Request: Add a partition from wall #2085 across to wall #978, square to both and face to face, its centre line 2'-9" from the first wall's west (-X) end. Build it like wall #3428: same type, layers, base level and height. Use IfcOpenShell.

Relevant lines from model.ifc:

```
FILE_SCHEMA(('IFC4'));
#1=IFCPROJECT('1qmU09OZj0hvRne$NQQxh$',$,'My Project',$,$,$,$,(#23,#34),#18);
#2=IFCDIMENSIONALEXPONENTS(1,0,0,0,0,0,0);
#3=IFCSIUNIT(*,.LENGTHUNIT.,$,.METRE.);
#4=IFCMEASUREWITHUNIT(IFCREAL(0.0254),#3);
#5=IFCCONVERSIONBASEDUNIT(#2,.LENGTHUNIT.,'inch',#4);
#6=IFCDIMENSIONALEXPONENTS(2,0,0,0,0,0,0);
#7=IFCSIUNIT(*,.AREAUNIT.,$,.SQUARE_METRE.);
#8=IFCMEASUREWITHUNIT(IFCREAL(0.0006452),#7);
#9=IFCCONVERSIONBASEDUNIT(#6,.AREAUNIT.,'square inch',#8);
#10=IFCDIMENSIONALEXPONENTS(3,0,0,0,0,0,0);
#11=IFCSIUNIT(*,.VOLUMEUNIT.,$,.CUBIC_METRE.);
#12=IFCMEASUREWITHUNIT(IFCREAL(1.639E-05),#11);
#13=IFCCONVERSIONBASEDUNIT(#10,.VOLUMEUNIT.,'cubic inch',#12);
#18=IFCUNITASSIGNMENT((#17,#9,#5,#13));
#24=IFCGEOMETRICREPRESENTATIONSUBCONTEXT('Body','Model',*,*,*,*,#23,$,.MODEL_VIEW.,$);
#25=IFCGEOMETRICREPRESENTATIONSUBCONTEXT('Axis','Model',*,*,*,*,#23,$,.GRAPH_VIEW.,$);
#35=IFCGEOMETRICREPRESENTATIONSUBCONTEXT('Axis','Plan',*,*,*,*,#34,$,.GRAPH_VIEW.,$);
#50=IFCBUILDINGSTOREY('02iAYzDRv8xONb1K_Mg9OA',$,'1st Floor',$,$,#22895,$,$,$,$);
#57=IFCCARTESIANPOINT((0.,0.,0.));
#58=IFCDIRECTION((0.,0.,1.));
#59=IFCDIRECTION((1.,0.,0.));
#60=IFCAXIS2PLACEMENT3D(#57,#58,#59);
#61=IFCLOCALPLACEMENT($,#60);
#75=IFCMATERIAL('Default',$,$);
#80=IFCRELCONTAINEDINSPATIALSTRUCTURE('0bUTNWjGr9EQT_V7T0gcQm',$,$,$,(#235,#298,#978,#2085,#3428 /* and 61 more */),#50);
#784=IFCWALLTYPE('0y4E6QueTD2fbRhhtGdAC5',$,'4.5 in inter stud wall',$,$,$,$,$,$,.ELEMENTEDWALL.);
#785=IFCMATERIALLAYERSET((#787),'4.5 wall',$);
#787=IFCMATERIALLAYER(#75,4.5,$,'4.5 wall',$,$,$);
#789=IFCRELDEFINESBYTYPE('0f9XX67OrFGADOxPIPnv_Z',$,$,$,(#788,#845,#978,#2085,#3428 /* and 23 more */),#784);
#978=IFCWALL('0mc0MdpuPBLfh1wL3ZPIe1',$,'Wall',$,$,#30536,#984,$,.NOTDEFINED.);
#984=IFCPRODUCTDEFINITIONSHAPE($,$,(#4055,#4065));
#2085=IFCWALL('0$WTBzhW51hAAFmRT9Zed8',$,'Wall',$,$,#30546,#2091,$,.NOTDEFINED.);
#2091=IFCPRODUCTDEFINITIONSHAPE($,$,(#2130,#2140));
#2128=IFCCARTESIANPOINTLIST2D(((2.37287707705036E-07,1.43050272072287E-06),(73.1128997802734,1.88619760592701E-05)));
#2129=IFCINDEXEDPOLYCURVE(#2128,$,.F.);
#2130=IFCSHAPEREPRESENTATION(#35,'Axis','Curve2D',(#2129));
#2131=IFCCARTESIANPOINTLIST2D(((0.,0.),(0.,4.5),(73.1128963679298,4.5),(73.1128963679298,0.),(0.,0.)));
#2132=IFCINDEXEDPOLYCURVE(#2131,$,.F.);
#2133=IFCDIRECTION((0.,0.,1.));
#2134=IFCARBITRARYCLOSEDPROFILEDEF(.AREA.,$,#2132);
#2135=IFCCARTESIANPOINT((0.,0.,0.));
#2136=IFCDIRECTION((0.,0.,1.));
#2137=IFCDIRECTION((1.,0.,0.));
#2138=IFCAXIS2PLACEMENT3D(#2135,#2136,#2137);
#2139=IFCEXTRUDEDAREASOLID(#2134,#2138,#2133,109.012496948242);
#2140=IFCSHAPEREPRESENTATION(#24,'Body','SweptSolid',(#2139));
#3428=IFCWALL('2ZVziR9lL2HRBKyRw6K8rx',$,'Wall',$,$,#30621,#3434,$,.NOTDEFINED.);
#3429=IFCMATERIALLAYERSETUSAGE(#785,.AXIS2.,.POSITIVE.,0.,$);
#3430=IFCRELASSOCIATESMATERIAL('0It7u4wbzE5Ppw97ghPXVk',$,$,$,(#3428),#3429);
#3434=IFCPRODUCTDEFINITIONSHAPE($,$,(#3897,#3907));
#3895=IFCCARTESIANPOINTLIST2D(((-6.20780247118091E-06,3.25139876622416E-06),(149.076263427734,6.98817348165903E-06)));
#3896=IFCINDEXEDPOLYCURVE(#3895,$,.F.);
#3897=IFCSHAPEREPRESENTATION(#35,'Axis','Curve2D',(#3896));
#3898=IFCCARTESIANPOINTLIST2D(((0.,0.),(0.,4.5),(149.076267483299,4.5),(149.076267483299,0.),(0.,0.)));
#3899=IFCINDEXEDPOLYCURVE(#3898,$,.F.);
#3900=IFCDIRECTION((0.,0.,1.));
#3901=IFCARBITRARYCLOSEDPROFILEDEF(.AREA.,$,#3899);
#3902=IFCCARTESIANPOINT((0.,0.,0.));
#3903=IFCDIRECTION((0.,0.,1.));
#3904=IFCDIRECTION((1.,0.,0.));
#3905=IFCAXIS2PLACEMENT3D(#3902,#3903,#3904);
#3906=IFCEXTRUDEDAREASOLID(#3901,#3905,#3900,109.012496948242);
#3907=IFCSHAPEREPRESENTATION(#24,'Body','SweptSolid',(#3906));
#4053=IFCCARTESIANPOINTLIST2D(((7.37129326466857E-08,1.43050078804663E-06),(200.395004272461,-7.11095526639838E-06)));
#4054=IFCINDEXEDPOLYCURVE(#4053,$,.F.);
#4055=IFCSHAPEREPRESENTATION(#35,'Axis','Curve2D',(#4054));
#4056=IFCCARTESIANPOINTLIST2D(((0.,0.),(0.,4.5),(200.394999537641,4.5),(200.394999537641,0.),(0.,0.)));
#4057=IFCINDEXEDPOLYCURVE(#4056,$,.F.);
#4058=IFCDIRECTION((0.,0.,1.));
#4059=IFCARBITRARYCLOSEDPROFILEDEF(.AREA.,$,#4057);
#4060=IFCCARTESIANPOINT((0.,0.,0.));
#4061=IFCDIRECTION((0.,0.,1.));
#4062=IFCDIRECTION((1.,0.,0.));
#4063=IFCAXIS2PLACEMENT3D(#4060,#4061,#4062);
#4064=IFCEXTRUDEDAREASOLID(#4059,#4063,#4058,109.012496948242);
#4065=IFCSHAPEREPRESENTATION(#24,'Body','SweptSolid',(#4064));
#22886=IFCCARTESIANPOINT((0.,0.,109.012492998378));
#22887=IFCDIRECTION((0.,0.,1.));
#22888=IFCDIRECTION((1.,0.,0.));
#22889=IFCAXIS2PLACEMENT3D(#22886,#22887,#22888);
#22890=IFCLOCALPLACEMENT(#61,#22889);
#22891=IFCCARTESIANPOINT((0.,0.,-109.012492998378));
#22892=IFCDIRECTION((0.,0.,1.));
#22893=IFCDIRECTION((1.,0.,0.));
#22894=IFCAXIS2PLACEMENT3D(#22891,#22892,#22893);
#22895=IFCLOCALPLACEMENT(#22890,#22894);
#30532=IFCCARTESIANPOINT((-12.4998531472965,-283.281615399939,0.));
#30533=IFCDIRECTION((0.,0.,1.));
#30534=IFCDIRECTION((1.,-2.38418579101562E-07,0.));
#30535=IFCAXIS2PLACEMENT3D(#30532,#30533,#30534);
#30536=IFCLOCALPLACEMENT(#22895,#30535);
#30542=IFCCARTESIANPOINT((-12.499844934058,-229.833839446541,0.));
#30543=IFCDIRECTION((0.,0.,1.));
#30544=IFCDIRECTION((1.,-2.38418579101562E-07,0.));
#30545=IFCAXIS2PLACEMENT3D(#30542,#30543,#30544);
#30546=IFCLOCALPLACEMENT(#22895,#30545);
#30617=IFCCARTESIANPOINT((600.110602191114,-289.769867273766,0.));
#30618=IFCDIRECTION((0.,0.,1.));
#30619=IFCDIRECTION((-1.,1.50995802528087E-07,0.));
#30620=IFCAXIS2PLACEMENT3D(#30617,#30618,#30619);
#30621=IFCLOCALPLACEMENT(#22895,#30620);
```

```python
import numpy as np
import ifcopenshell
import ifcopenshell.api.geometry
import ifcopenshell.api.material
import ifcopenshell.api.pset
import ifcopenshell.api.root
import ifcopenshell.api.spatial
import ifcopenshell.api.type
import ifcopenshell.geom
import ifcopenshell.util.element
import ifcopenshell.util.placement
import ifcopenshell.util.representation
import ifcopenshell.util.shape
import ifcopenshell.util.unit

model = ifcopenshell.open("model.ifc")
unit_scale = ifcopenshell.util.unit.calculate_unit_scale(model)
settings = ifcopenshell.geom.settings()
settings.set("use-world-coords", True)

start_wall = model.by_id(2085)
end_wall = model.by_guid("0mc0MdpuPBLfh1wL3ZPIe1")
like = model.by_id(3428)
matrix = ifcopenshell.util.placement.get_local_placement(start_wall.ObjectPlacement)
matrix[:3, 3] *= unit_scale


def extent(element):
    """Bounding box in the first wall's axes, in metres."""
    shape = ifcopenshell.geom.create_shape(settings, element)
    points = (ifcopenshell.util.shape.get_vertices(shape.geometry) - matrix[:3, 3]) @ matrix[:3, :3]
    return points.min(axis=0), points.max(axis=0)


y_start = extent(start_wall)[0][1]
y_end = extent(end_wall)[1][1]
like_min, like_max = extent(like)
length, height = float(abs(y_end - y_start)), float(like_max[2] - like_min[2])
layer_set = ifcopenshell.util.element.get_material(like, should_skip_usage=True)
thickness = sum(layer.LayerThickness for layer in layer_set.MaterialLayers) * unit_scale

wall = ifcopenshell.api.root.create_entity(model, ifc_class="IfcWall", name="New partition")
storey = ifcopenshell.util.element.get_container(like)
ifcopenshell.api.spatial.assign_container(model, products=[wall], relating_structure=storey)
ifcopenshell.api.type.assign_type(
    model, related_objects=[wall], relating_type=ifcopenshell.util.element.get_type(like), should_map_representations=False
)
rel = ifcopenshell.api.material.assign_material(
    model, products=[wall], type="IfcMaterialLayerSetUsage", material=layer_set
)
rel.RelatingMaterial.OffsetFromReferenceLine = -thickness / 2 / unit_scale
pset = ifcopenshell.api.pset.add_pset(model, product=wall, name="Pset_WallCommon")
ifcopenshell.api.pset.edit_pset(model, pset=pset, properties={"IsExternal": False, "LoadBearing": False})

# The axis runs down the middle of the wall.
axis = ifcopenshell.api.geometry.add_axis_representation(
    model, context=ifcopenshell.util.representation.get_context(model, "Model", "Axis"), axis=[(0.0, 0.0), (length, 0.0)]
)
body = ifcopenshell.api.geometry.add_wall_representation(
    model,
    context=ifcopenshell.util.representation.get_context(model, "Model", "Body", "MODEL_VIEW"),
    length=length,
    height=height,
    thickness=thickness,
    offset=-thickness / 2,
)
for representation in (axis, body):
    ifcopenshell.api.geometry.assign_representation(model, product=wall, representation=representation)

placement = matrix @ ifcopenshell.util.placement.rotation(-90, "Z")
placement[:, 3] = matrix @ np.array([extent(start_wall)[0][0] + 0.8382, y_start, like_min[2], 1.0])
ifcopenshell.api.geometry.edit_object_placement(model, product=wall, matrix=placement)

print(f"partition {length:.3f} m long, {height:.3f} m high, {thickness:.3f} m thick")

model.write("model_edited.ifc")
```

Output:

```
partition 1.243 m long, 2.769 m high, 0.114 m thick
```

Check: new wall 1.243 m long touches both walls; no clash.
